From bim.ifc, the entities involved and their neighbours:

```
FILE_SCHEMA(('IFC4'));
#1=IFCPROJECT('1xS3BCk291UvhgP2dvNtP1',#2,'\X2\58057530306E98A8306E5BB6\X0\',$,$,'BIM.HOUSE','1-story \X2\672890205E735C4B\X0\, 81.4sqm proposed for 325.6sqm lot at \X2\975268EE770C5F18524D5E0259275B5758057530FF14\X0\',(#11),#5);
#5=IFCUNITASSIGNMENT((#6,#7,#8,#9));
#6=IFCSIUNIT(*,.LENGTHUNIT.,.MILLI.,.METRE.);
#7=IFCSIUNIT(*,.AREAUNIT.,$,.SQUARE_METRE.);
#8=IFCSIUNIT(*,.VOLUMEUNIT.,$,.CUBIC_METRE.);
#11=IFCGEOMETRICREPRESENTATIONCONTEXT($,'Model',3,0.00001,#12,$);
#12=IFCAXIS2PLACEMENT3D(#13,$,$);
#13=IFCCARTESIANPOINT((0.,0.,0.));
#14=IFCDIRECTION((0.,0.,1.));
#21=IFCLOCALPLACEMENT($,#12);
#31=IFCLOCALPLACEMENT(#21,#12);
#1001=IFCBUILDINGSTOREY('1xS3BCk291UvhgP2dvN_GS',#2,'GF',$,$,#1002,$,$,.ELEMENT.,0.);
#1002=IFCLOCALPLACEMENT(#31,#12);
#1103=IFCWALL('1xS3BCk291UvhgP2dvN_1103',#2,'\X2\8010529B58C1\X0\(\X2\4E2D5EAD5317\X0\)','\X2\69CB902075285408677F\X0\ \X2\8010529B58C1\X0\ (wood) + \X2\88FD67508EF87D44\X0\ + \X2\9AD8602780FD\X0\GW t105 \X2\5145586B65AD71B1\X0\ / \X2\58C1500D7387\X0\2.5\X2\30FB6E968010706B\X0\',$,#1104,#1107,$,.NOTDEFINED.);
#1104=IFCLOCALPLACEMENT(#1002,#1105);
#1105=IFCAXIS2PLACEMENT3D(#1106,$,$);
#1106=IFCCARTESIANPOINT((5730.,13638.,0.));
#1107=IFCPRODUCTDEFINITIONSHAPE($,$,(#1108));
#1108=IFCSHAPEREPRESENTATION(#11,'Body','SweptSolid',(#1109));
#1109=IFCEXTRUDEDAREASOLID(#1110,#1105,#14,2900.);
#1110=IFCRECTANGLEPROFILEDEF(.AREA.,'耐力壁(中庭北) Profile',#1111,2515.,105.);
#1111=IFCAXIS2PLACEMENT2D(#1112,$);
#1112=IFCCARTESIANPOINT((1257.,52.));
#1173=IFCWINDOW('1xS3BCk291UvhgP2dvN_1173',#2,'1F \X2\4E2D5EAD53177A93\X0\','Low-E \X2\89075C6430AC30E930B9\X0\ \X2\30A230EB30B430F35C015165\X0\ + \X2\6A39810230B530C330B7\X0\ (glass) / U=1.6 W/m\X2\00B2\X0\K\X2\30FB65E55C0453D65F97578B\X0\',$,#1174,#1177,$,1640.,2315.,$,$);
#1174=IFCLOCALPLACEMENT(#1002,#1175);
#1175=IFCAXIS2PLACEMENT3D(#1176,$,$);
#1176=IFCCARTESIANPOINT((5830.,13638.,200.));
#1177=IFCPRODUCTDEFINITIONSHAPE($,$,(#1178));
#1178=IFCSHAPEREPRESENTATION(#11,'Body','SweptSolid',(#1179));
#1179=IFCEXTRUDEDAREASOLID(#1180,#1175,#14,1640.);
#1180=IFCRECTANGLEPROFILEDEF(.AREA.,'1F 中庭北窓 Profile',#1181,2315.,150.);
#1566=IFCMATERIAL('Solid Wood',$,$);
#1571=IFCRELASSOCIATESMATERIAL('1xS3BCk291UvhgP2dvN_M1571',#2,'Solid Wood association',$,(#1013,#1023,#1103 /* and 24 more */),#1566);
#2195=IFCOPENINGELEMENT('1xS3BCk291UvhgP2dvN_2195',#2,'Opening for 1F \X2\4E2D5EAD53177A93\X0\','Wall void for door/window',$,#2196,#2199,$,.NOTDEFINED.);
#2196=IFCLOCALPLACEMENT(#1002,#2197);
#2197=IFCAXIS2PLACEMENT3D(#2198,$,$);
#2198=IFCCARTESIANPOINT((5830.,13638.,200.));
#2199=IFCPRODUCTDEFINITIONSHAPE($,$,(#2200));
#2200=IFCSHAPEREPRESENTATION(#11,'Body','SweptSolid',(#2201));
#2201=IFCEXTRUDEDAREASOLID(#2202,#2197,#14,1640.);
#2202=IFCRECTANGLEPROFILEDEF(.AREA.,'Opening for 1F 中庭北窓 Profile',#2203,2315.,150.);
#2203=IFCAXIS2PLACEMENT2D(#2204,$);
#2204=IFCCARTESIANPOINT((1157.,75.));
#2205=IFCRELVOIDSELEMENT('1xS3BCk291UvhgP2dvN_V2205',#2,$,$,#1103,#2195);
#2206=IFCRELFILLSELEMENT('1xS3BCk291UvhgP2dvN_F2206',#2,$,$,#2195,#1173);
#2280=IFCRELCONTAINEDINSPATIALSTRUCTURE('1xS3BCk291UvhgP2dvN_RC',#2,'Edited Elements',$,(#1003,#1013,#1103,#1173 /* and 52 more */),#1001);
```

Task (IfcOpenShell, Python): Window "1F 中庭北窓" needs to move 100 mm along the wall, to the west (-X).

```python
import ifcopenshell
import ifcopenshell.api.geometry
import ifcopenshell.util.placement
import ifcopenshell.util.unit

model = ifcopenshell.open("bim.ifc")
unit_scale = ifcopenshell.util.unit.calculate_unit_scale(model)

window = model.by_guid("1xS3BCk291UvhgP2dvN_1173")
opening = window.FillsVoids[0].RelatingOpeningElement
wall = opening.VoidsElements[0].RelatingBuildingElement

wall_matrix = ifcopenshell.util.placement.get_local_placement(wall.ObjectPlacement)
shift = wall_matrix[:3, 0] * -0.1 / unit_scale
before = ifcopenshell.util.placement.get_local_placement(window.ObjectPlacement)[:3, 3].copy()

# The window is not placed relative to its opening, so move both.
for product in (opening, window):
    matrix = ifcopenshell.util.placement.get_local_placement(product.ObjectPlacement)
    matrix[:3, 3] += shift
    ifcopenshell.api.geometry.edit_object_placement(model, product=product, matrix=matrix, is_si=False)

after = ifcopenshell.util.placement.get_local_placement(window.ObjectPlacement)[:3, 3]
print("window moved by", (after - before).round(3) + 0.0)

model.write("bim_v2.ifc")
```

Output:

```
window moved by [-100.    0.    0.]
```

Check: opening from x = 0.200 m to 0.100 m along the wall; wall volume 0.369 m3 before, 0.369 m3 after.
